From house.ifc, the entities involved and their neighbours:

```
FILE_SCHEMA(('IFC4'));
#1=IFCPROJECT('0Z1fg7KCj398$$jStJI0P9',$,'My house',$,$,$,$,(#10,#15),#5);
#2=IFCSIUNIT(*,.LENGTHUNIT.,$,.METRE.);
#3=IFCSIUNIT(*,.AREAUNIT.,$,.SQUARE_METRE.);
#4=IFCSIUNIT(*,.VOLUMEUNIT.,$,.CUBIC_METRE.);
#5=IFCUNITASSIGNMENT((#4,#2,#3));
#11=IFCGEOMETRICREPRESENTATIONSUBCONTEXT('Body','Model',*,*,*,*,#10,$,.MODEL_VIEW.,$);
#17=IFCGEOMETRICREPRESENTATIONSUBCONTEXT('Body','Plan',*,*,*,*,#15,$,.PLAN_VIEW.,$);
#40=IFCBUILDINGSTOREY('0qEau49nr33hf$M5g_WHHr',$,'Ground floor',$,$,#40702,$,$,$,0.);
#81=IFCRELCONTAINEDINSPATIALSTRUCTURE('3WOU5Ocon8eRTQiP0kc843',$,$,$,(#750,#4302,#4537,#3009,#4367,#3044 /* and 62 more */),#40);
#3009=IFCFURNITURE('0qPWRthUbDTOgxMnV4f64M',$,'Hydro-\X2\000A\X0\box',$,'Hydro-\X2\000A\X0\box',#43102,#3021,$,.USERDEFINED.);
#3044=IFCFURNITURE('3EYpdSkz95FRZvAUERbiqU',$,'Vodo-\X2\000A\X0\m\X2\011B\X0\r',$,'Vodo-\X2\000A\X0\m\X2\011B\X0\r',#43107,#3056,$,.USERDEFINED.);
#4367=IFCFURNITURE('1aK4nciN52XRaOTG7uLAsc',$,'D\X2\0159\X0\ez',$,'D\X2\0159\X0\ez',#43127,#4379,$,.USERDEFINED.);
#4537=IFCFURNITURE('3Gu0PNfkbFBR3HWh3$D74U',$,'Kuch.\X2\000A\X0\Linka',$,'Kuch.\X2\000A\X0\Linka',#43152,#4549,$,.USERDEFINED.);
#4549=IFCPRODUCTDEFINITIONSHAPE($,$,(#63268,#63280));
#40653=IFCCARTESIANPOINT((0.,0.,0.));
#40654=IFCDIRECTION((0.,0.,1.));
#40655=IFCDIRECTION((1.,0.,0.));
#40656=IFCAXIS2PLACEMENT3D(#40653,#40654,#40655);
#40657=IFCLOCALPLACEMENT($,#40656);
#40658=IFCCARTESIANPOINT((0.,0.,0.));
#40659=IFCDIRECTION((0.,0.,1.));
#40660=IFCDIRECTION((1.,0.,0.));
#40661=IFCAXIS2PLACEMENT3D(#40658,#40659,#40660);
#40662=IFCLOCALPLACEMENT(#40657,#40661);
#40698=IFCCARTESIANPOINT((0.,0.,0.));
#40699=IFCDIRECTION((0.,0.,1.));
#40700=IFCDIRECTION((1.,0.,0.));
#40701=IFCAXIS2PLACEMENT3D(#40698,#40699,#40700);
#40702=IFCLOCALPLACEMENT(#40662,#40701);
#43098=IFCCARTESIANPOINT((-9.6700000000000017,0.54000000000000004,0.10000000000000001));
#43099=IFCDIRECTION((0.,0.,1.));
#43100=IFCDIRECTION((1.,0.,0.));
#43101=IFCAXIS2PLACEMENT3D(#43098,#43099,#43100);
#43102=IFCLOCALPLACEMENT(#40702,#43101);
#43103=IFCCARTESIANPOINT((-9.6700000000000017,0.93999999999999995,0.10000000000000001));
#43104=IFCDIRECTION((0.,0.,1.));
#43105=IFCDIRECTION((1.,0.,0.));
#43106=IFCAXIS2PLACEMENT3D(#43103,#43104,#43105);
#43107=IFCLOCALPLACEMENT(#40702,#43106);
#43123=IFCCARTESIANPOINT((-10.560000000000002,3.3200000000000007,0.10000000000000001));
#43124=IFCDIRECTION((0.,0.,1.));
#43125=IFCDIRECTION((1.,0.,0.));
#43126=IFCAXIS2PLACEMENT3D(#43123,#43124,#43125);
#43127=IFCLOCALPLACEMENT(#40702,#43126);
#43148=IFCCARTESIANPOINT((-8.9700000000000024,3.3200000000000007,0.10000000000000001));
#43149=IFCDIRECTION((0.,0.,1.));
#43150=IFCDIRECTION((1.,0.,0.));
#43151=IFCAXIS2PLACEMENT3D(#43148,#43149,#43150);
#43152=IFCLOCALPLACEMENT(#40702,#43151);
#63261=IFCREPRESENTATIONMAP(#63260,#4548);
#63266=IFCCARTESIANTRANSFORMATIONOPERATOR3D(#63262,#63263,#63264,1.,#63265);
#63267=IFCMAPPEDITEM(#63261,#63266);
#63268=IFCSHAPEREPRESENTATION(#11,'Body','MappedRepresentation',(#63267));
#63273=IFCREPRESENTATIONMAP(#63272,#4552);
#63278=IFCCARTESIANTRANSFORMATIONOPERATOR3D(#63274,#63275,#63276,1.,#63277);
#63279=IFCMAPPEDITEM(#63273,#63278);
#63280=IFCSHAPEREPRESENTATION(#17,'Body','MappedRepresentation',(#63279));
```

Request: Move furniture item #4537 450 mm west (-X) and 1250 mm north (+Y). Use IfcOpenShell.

```python
import ifcopenshell
import ifcopenshell.api.geometry
import ifcopenshell.util.placement

model = ifcopenshell.open("house.ifc")

item = model.by_guid("3Gu0PNfkbFBR3HWh3$D74U")
matrix = ifcopenshell.util.placement.get_local_placement(item.ObjectPlacement)
matrix[0, 3] -= 0.45
matrix[1, 3] += 1.25
ifcopenshell.api.geometry.edit_object_placement(model, product=item, matrix=matrix, is_si=False)

print(ifcopenshell.util.placement.get_local_placement(item.ObjectPlacement).round(3) + 0.0)

model.write("house_rev.ifc")
```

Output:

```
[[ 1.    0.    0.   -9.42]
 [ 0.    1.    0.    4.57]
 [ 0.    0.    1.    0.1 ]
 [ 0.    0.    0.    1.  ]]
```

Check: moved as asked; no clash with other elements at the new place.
